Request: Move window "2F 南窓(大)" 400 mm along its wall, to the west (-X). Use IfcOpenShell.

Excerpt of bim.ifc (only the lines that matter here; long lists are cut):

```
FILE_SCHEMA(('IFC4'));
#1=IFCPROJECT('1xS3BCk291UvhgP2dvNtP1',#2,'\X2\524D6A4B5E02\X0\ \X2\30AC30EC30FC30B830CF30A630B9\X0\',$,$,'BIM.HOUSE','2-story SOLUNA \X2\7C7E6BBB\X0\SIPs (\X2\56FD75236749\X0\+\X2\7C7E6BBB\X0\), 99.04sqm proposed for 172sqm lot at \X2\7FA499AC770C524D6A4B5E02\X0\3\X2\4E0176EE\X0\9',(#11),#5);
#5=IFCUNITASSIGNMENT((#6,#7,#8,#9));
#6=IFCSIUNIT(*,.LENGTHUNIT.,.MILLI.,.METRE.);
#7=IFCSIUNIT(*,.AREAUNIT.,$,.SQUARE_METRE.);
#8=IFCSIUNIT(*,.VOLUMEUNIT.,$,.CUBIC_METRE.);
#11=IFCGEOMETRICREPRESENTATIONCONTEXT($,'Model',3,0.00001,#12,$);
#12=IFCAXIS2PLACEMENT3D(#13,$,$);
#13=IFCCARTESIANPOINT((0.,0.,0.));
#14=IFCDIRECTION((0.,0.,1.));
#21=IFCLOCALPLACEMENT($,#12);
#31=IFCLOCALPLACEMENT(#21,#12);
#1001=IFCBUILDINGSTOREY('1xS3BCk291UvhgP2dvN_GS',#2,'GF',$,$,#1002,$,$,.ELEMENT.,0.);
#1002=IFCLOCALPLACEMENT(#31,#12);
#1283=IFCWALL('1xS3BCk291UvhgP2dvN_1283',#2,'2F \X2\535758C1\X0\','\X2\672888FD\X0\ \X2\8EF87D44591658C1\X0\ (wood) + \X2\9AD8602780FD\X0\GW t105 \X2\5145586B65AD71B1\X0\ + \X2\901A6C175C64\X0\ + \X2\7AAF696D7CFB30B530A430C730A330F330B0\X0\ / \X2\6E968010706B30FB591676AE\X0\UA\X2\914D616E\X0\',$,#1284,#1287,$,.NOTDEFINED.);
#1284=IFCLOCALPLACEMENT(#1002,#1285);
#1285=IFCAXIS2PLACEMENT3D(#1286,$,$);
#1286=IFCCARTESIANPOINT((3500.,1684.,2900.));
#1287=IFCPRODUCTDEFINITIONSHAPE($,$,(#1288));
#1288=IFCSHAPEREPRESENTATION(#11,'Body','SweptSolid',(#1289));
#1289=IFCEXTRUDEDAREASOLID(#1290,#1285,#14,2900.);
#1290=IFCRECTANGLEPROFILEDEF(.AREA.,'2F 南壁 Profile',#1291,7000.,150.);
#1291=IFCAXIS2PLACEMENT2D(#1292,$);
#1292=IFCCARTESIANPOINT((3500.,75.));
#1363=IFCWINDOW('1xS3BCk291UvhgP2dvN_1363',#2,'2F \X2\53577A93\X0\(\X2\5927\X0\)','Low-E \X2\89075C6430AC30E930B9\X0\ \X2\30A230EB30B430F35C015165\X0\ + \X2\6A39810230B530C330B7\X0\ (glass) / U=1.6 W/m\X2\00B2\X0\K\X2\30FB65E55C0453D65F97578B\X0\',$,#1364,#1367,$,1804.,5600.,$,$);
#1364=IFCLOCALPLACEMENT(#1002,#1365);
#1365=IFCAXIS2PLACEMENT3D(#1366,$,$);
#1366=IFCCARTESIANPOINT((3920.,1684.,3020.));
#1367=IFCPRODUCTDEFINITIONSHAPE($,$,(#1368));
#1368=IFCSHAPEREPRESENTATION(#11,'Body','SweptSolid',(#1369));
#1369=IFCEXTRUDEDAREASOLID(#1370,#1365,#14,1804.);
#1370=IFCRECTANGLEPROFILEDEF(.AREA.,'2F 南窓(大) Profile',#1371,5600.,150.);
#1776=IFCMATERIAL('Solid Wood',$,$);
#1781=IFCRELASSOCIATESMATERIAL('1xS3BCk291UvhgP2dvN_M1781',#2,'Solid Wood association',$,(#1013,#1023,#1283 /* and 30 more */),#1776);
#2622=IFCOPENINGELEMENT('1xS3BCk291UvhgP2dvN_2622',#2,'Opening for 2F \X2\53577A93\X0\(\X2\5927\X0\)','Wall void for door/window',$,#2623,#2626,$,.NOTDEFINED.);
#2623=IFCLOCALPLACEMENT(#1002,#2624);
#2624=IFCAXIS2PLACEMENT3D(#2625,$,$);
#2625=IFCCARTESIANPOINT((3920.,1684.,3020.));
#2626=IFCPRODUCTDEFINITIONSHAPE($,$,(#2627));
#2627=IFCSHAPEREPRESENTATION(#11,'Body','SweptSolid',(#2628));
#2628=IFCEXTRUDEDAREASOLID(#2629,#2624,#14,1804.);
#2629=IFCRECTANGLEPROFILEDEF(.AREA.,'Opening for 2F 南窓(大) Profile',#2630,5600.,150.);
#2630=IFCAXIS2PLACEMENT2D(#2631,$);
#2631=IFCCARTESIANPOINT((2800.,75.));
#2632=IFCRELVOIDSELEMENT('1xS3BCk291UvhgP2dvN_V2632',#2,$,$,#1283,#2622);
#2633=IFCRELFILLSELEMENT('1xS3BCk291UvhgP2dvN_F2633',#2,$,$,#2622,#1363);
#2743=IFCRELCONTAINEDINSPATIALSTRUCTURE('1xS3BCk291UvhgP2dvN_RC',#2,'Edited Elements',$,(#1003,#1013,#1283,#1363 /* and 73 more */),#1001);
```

```python
import ifcopenshell
import ifcopenshell.api.geometry
import ifcopenshell.util.placement
import ifcopenshell.util.unit

model = ifcopenshell.open("bim.ifc")
unit_scale = ifcopenshell.util.unit.calculate_unit_scale(model)

window = model.by_guid("1xS3BCk291UvhgP2dvN_1363")
opening = window.FillsVoids[0].RelatingOpeningElement
wall = opening.VoidsElements[0].RelatingBuildingElement

wall_matrix = ifcopenshell.util.placement.get_local_placement(wall.ObjectPlacement)
shift = wall_matrix[:3, 0] * -0.4 / unit_scale
before = ifcopenshell.util.placement.get_local_placement(window.ObjectPlacement)[:3, 3].copy()

# The window is not placed relative to its opening, so move both.
for product in (opening, window):
    matrix = ifcopenshell.util.placement.get_local_placement(product.ObjectPlacement)
    matrix[:3, 3] += shift
    ifcopenshell.api.geometry.edit_object_placement(model, product=product, matrix=matrix, is_si=False)

after = ifcopenshell.util.placement.get_local_placement(window.ObjectPlacement)[:3, 3]
print("window moved by", (after - before).round(3) + 0.0)

model.write("bim-out.ifc")
```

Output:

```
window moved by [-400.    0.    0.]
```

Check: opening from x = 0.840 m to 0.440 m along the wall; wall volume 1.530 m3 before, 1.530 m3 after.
